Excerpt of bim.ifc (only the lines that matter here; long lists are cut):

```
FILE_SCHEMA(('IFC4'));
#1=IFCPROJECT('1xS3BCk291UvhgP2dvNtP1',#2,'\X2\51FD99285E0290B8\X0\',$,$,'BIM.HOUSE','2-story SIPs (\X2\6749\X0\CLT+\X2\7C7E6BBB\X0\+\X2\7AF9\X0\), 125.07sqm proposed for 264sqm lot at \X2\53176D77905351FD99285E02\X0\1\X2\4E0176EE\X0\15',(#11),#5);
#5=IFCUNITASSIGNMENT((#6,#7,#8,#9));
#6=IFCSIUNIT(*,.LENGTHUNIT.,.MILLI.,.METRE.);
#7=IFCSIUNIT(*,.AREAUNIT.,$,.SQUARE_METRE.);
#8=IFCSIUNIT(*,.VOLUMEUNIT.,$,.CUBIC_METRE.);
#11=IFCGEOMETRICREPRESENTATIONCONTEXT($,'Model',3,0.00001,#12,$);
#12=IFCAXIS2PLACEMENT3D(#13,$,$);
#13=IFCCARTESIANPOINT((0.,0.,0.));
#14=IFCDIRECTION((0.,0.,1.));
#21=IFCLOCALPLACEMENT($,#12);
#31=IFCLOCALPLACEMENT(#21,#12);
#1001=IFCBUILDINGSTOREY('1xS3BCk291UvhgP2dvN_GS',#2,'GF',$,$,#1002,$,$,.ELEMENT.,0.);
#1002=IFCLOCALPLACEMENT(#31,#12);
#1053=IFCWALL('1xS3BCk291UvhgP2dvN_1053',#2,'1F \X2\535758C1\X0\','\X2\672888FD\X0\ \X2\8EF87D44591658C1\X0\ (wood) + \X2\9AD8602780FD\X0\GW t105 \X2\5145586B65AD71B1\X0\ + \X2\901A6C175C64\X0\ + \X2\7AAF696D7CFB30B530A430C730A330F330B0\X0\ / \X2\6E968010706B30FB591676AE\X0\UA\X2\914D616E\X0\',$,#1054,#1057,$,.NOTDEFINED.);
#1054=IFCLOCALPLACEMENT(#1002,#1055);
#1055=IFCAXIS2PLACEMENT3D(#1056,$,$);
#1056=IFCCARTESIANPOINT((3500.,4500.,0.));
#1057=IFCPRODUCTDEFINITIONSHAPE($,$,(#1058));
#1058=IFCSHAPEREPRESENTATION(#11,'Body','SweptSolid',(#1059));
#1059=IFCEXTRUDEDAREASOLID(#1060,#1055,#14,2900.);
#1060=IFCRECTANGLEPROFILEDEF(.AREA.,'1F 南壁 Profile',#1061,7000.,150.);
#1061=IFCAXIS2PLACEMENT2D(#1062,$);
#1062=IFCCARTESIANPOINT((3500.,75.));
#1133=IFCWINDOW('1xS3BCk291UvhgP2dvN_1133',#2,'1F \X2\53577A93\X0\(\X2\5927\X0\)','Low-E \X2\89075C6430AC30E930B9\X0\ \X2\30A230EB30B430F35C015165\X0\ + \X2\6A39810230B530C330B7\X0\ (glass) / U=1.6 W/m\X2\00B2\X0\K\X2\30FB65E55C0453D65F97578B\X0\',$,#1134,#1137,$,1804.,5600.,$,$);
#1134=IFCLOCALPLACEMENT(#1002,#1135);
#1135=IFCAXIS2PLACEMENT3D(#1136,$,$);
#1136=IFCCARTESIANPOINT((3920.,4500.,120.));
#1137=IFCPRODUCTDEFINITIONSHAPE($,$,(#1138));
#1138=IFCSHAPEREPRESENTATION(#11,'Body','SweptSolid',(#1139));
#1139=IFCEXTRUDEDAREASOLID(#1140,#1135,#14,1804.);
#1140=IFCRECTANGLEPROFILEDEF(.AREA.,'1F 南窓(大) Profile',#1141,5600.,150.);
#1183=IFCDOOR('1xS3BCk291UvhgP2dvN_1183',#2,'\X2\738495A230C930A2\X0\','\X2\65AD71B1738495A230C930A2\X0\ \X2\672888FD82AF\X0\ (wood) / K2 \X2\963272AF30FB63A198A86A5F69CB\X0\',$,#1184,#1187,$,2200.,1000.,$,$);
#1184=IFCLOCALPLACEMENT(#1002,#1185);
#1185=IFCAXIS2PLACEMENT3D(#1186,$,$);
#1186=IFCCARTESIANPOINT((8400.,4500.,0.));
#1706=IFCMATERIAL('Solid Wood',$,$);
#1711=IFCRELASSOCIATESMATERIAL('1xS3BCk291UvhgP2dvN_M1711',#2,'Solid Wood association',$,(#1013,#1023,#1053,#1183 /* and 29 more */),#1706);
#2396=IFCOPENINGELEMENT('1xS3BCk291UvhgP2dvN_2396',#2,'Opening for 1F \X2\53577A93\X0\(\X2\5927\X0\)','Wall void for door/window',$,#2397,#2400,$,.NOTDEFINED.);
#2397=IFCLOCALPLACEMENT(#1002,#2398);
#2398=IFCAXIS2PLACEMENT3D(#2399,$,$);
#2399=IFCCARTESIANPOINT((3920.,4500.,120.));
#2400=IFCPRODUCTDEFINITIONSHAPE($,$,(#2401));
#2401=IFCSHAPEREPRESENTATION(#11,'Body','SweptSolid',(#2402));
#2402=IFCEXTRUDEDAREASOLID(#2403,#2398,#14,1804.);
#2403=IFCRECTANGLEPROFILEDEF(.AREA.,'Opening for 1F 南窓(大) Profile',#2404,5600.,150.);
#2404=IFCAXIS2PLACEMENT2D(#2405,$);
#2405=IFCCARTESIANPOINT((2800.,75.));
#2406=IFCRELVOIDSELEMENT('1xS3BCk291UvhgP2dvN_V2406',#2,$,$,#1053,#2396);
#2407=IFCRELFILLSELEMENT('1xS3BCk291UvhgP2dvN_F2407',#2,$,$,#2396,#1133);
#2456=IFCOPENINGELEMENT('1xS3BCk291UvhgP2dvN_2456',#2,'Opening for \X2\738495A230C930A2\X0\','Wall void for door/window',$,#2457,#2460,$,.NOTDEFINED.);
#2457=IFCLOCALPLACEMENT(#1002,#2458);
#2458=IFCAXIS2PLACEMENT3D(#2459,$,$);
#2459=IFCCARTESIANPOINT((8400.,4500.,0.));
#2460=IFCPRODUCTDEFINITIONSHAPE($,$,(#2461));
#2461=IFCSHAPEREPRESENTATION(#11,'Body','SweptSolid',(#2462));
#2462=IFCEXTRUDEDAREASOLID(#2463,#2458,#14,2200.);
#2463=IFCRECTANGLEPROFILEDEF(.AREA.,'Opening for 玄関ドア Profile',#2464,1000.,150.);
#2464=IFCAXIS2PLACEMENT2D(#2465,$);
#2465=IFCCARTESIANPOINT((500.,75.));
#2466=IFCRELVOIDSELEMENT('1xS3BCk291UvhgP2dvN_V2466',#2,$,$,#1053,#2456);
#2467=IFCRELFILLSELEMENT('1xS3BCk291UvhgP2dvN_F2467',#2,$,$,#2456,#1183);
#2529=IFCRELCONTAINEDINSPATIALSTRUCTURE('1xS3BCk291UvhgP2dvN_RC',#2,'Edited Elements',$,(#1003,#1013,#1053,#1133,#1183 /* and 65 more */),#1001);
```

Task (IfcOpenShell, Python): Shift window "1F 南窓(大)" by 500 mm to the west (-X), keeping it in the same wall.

```python
import ifcopenshell
import ifcopenshell.api.geometry
import ifcopenshell.util.placement
import ifcopenshell.util.unit

model = ifcopenshell.open("bim.ifc")
unit_scale = ifcopenshell.util.unit.calculate_unit_scale(model)

window = model.by_id(1133)
opening = window.FillsVoids[0].RelatingOpeningElement
wall = opening.VoidsElements[0].RelatingBuildingElement

wall_matrix = ifcopenshell.util.placement.get_local_placement(wall.ObjectPlacement)
shift = wall_matrix[:3, 0] * -0.5 / unit_scale
before = ifcopenshell.util.placement.get_local_placement(window.ObjectPlacement)[:3, 3].copy()

# The window is not placed relative to its opening, so move both.
for product in (opening, window):
    matrix = ifcopenshell.util.placement.get_local_placement(product.ObjectPlacement)
    matrix[:3, 3] += shift
    ifcopenshell.api.geometry.edit_object_placement(model, product=product, matrix=matrix, is_si=False)

after = ifcopenshell.util.placement.get_local_placement(window.ObjectPlacement)[:3, 3]
print("window moved by", (after - before).round(3) + 0.0)

model.write("bim_updated.ifc")
```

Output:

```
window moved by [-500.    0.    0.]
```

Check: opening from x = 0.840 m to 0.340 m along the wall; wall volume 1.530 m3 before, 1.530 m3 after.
